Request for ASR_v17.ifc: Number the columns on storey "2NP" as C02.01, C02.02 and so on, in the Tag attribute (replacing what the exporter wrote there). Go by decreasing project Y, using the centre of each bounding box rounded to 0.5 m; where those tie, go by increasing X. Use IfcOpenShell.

First a look at what the model holds.

```python
import ifcopenshell
import ifcopenshell.util.element
import ifcopenshell.util.placement

model = ifcopenshell.open("ASR_v17.ifc")
print(model.schema)
storey = next(s for s in model.by_type("IfcBuildingStorey") if s.Name == "2NP")
columns = [e for e in ifcopenshell.util.element.get_decomposition(storey) if e.is_a("IfcColumn")]
for e in sorted(columns, key=lambda e: e.id()):
    origin = ifcopenshell.util.placement.get_local_placement(e.ObjectPlacement)[:3, 3]
    print(e.id(), e.Tag, e.Name, origin.round(2) + 0.0, sep=" | ")
```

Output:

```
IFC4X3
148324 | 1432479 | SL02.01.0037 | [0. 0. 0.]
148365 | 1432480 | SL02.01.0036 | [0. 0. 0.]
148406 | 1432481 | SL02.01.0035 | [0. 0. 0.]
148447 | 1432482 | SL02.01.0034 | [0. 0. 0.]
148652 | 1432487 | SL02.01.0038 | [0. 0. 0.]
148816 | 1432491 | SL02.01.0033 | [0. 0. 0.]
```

```python
import ifcopenshell
import ifcopenshell.geom
import ifcopenshell.util.element
import ifcopenshell.util.shape

model = ifcopenshell.open("ASR_v17.ifc")
settings = ifcopenshell.geom.settings()
settings.set("use-world-coords", True)


def centre(element):
    shape = ifcopenshell.geom.create_shape(settings, element)
    return ifcopenshell.util.shape.get_bbox_centroid(shape.geometry)


storey = next(s for s in model.by_type("IfcBuildingStorey") if s.Name == "2NP")
columns = [e for e in ifcopenshell.util.element.get_decomposition(storey) if e.is_a("IfcColumn")]

# Insertion points can sit at a corner or the storey origin, so sort by the geometry (in metres).
centres = {e: centre(e) for e in columns}
columns.sort(key=lambda e: (-round(centres[e][1] / 0.5), centres[e][0]))

for i, e in enumerate(columns, start=1):
    number = f"C02.{i:02d}"
    e.Tag = number
    print(e.id(), number)

model.write("ASR_v17-out.ifc")
```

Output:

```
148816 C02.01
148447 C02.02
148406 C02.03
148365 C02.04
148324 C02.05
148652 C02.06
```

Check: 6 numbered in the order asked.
